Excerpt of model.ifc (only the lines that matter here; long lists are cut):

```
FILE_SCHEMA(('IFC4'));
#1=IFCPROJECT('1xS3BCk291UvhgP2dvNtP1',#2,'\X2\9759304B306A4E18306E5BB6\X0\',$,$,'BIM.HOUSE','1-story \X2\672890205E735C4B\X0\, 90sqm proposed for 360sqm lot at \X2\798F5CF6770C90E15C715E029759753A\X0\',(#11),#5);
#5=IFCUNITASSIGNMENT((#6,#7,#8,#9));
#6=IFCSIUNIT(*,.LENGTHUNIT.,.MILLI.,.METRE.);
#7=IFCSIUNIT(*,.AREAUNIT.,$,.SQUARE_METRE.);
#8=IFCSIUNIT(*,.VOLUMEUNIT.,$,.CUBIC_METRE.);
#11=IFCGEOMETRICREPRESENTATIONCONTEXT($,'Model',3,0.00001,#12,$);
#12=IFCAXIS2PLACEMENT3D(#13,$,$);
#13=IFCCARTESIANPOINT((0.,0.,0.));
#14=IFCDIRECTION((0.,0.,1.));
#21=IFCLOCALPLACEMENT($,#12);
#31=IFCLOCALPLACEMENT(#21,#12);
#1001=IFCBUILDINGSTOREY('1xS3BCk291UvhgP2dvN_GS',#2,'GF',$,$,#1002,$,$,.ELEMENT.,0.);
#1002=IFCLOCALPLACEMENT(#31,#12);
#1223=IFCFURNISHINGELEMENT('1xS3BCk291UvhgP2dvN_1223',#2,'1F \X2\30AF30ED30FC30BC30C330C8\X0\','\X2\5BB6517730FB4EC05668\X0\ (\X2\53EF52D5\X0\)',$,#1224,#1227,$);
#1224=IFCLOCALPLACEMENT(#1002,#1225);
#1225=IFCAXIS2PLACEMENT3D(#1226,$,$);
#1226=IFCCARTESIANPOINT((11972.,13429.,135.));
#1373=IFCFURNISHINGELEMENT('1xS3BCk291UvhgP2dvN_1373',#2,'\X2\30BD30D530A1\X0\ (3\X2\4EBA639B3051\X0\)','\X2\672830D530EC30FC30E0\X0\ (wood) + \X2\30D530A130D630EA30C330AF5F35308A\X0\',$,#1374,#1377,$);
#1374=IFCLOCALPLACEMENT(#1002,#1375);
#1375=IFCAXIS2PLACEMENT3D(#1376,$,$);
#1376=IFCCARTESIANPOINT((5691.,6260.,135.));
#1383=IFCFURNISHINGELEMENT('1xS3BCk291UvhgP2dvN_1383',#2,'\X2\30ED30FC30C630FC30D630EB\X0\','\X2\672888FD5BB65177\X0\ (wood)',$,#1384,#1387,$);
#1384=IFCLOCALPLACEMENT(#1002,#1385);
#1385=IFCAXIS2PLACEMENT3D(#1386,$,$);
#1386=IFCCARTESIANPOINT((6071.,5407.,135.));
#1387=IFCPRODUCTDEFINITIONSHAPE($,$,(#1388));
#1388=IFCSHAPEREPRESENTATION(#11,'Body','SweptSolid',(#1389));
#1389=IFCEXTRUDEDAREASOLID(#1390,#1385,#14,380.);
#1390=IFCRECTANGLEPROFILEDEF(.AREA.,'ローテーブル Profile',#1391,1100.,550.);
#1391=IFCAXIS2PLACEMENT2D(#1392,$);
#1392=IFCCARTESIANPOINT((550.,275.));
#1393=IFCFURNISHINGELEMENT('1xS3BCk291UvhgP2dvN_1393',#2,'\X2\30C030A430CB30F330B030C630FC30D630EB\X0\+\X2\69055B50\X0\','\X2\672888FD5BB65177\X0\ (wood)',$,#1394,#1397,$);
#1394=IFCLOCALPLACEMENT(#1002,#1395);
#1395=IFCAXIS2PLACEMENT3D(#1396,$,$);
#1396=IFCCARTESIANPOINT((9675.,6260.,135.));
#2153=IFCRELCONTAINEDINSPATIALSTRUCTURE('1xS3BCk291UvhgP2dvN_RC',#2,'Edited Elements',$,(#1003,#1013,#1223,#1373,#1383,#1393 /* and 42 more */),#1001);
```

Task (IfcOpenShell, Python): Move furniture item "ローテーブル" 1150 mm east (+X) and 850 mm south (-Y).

```python
import ifcopenshell
import ifcopenshell.api.geometry
import ifcopenshell.util.placement

model = ifcopenshell.open("model.ifc")

item = model.by_id(1383)
matrix = ifcopenshell.util.placement.get_local_placement(item.ObjectPlacement)
matrix[0, 3] += 1150.0
matrix[1, 3] -= 850.0
ifcopenshell.api.geometry.edit_object_placement(model, product=item, matrix=matrix, is_si=False)

print(ifcopenshell.util.placement.get_local_placement(item.ObjectPlacement).round(3) + 0.0)

model.write("model_v2.ifc")
```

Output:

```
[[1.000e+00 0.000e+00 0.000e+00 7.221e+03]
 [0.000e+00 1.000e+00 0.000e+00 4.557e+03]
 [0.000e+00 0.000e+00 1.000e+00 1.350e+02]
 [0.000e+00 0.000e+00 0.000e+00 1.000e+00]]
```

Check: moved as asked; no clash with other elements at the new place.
